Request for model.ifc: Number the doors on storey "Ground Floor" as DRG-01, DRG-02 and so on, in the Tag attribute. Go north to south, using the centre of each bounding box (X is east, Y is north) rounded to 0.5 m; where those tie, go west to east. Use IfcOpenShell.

First a look at what the model holds.

```python
import ifcopenshell
import ifcopenshell.util.element
import ifcopenshell.util.placement

model = ifcopenshell.open("model.ifc")
print(model.schema)
storey = next(s for s in model.by_type("IfcBuildingStorey") if s.Name == "Ground Floor")
doors = [e for e in ifcopenshell.util.element.get_decomposition(storey) if e.is_a("IfcDoor")]
for e in sorted(doors, key=lambda e: e.id()):
    origin = ifcopenshell.util.placement.get_local_placement(e.ObjectPlacement)[:3, 3]
    print(e.id(), e.Tag, e.Name, origin.round(2) + 0.0, sep=" | ")
```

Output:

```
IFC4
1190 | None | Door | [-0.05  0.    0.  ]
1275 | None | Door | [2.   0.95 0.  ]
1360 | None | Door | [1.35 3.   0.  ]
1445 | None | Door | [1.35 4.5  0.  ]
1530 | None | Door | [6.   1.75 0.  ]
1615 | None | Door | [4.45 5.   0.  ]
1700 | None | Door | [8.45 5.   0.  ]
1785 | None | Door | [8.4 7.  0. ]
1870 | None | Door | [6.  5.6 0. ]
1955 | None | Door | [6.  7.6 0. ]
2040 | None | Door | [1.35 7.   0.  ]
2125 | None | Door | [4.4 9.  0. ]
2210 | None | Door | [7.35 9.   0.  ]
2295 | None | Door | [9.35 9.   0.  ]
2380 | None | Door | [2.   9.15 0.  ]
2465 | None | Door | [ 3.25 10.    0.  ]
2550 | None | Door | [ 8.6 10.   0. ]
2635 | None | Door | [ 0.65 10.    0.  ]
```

```python
import ifcopenshell
import ifcopenshell.geom
import ifcopenshell.util.element
import ifcopenshell.util.shape

model = ifcopenshell.open("model.ifc")
settings = ifcopenshell.geom.settings()
settings.set("use-world-coords", True)


def centre(element):
    shape = ifcopenshell.geom.create_shape(settings, element)
    return ifcopenshell.util.shape.get_bbox_centroid(shape.geometry)


storey = next(s for s in model.by_type("IfcBuildingStorey") if s.Name == "Ground Floor")
doors = [e for e in ifcopenshell.util.element.get_decomposition(storey) if e.is_a("IfcDoor")]

# Insertion points can sit at a corner or the storey origin, so sort by the geometry (in metres).
centres = {e: centre(e) for e in doors}
doors.sort(key=lambda e: (-round(centres[e][1] / 0.5), centres[e][0]))

for i, e in enumerate(doors, start=1):
    number = f"DRG-{i:02d}"
    e.Tag = number
    print(e.id(), number)

model.write("model_updated.ifc")
```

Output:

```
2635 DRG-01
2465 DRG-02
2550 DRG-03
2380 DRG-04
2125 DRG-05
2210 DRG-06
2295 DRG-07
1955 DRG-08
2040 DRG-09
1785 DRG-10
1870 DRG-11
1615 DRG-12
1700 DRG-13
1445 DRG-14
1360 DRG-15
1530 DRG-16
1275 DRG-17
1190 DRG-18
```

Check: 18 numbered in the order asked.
